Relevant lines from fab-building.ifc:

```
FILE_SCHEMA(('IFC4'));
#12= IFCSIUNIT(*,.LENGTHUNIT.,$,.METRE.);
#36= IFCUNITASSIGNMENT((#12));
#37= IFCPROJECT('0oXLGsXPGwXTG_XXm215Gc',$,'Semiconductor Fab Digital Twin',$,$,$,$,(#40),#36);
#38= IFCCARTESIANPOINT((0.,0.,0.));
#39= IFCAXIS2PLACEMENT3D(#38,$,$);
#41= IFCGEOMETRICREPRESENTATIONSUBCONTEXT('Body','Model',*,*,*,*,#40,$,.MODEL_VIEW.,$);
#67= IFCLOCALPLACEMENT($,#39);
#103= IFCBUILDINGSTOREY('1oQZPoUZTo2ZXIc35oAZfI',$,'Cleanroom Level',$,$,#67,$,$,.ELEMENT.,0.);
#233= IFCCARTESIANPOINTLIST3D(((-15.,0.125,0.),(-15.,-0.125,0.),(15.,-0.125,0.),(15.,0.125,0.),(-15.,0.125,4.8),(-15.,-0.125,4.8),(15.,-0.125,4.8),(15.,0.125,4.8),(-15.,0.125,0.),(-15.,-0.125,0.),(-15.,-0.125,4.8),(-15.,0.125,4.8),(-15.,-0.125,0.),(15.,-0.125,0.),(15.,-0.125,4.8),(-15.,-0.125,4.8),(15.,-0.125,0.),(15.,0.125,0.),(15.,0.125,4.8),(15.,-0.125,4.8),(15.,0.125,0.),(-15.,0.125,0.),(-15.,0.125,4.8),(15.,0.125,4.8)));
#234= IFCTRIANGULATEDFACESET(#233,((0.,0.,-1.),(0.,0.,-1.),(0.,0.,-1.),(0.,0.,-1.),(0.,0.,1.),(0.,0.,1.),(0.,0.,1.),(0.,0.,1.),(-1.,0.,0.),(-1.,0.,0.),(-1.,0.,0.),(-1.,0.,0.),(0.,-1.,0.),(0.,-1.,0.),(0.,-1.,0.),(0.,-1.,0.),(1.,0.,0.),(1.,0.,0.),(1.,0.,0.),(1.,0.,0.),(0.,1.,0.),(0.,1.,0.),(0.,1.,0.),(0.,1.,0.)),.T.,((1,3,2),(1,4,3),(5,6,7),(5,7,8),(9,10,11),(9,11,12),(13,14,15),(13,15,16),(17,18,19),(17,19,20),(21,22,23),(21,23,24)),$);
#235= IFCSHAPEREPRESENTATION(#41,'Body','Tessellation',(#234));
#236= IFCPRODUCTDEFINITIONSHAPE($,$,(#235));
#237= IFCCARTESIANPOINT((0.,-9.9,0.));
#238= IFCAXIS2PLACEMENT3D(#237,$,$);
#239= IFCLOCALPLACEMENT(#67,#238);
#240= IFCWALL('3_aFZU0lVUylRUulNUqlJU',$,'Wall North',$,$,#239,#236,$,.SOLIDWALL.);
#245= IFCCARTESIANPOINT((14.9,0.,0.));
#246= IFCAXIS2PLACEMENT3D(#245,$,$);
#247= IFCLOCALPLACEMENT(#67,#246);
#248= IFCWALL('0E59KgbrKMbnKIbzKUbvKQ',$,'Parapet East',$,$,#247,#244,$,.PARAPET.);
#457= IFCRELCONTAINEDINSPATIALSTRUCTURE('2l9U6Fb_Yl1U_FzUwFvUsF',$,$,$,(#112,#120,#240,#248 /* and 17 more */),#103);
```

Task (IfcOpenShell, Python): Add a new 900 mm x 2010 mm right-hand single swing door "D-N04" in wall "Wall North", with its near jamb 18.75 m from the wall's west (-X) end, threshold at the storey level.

```python
import numpy as np
import ifcopenshell
import ifcopenshell.api.feature
import ifcopenshell.api.geometry
import ifcopenshell.api.root
import ifcopenshell.api.spatial
import ifcopenshell.geom
import ifcopenshell.util.element
import ifcopenshell.util.placement
import ifcopenshell.util.representation
import ifcopenshell.util.shape
import ifcopenshell.util.unit

model = ifcopenshell.open("fab-building.ifc")
unit_scale = ifcopenshell.util.unit.calculate_unit_scale(model)
settings = ifcopenshell.geom.settings()


def volume(element):
    """Net volume in cubic metres, openings subtracted."""
    shape = ifcopenshell.geom.create_shape(settings, element)
    return ifcopenshell.util.shape.get_volume(shape.geometry)


wall = model.by_guid("3_aFZU0lVUylRUulNUqlJU")
storey = ifcopenshell.util.element.get_container(wall, ifc_class="IfcBuildingStorey")
context = ifcopenshell.util.representation.get_context(model, "Model", "Body", "MODEL_VIEW")
before = volume(wall)

width, height, from_end, sill = 0.9, 2.01, 18.75, 0.0  # metres

# The wall runs along its own X axis, and the end named is its -X end.
wall_shape = ifcopenshell.geom.create_shape(settings, wall)
x, y, z = ifcopenshell.util.shape.get_vertices(wall_shape.geometry).T
start = x.min() + from_end
face, thickness = float(y.min()), float(y.max() - y.min())
wall_matrix = ifcopenshell.util.placement.get_local_placement(wall.ObjectPlacement)
level = ifcopenshell.util.placement.get_local_placement(storey.ObjectPlacement)[2, 3]


def in_wall(x, y):
    """Placement at x, y metres in the wall's axes, at sill height."""
    matrix = wall_matrix.copy()
    matrix[:, 3] = wall_matrix @ np.array([x / unit_scale, y / unit_scale, 0.0, 1.0])
    matrix[2, 3] = level + sill / unit_scale
    return matrix


# Opening: a box that overshoots both wall faces by 50 mm.
opening = ifcopenshell.api.root.create_entity(model, ifc_class="IfcOpeningElement", predefined_type="OPENING")
box = ifcopenshell.api.geometry.add_wall_representation(
    model, context=context, length=width, height=height, thickness=thickness + 0.1
)
ifcopenshell.api.geometry.assign_representation(model, product=opening, representation=box)
ifcopenshell.api.geometry.edit_object_placement(model, product=opening, matrix=in_wall(start, face - 0.05), is_si=False)
ifcopenshell.api.feature.add_feature(model, feature=opening, element=wall)

door = ifcopenshell.api.root.create_entity(model, ifc_class="IfcDoor", name="D-N04", predefined_type="DOOR")
door.OverallWidth, door.OverallHeight = width / unit_scale, height / unit_scale
door.OperationType = "SINGLE_SWING_RIGHT"
body = ifcopenshell.api.geometry.add_door_representation(
    model,
    context=context,
    overall_width=door.OverallWidth,
    overall_height=door.OverallHeight,
    operation_type="SINGLE_SWING_RIGHT",
    lining_properties={"LiningDepth": thickness / unit_scale, "ThresholdDepth": thickness / unit_scale},
)
ifcopenshell.api.geometry.assign_representation(model, product=door, representation=body)
ifcopenshell.api.spatial.assign_container(model, products=[door], relating_structure=storey)
ifcopenshell.api.feature.add_filling(model, opening=opening, element=door)

# The lining spans the wall, so the door starts at the wall face.
ifcopenshell.api.geometry.edit_object_placement(model, product=door, matrix=in_wall(start, face), is_si=False)

after = volume(wall)

print(f"wall volume {before:.3f} -> {after:.3f} m3")

model.write("fab-building_edited.ifc")
```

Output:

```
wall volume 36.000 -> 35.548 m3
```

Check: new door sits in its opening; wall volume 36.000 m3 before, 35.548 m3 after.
